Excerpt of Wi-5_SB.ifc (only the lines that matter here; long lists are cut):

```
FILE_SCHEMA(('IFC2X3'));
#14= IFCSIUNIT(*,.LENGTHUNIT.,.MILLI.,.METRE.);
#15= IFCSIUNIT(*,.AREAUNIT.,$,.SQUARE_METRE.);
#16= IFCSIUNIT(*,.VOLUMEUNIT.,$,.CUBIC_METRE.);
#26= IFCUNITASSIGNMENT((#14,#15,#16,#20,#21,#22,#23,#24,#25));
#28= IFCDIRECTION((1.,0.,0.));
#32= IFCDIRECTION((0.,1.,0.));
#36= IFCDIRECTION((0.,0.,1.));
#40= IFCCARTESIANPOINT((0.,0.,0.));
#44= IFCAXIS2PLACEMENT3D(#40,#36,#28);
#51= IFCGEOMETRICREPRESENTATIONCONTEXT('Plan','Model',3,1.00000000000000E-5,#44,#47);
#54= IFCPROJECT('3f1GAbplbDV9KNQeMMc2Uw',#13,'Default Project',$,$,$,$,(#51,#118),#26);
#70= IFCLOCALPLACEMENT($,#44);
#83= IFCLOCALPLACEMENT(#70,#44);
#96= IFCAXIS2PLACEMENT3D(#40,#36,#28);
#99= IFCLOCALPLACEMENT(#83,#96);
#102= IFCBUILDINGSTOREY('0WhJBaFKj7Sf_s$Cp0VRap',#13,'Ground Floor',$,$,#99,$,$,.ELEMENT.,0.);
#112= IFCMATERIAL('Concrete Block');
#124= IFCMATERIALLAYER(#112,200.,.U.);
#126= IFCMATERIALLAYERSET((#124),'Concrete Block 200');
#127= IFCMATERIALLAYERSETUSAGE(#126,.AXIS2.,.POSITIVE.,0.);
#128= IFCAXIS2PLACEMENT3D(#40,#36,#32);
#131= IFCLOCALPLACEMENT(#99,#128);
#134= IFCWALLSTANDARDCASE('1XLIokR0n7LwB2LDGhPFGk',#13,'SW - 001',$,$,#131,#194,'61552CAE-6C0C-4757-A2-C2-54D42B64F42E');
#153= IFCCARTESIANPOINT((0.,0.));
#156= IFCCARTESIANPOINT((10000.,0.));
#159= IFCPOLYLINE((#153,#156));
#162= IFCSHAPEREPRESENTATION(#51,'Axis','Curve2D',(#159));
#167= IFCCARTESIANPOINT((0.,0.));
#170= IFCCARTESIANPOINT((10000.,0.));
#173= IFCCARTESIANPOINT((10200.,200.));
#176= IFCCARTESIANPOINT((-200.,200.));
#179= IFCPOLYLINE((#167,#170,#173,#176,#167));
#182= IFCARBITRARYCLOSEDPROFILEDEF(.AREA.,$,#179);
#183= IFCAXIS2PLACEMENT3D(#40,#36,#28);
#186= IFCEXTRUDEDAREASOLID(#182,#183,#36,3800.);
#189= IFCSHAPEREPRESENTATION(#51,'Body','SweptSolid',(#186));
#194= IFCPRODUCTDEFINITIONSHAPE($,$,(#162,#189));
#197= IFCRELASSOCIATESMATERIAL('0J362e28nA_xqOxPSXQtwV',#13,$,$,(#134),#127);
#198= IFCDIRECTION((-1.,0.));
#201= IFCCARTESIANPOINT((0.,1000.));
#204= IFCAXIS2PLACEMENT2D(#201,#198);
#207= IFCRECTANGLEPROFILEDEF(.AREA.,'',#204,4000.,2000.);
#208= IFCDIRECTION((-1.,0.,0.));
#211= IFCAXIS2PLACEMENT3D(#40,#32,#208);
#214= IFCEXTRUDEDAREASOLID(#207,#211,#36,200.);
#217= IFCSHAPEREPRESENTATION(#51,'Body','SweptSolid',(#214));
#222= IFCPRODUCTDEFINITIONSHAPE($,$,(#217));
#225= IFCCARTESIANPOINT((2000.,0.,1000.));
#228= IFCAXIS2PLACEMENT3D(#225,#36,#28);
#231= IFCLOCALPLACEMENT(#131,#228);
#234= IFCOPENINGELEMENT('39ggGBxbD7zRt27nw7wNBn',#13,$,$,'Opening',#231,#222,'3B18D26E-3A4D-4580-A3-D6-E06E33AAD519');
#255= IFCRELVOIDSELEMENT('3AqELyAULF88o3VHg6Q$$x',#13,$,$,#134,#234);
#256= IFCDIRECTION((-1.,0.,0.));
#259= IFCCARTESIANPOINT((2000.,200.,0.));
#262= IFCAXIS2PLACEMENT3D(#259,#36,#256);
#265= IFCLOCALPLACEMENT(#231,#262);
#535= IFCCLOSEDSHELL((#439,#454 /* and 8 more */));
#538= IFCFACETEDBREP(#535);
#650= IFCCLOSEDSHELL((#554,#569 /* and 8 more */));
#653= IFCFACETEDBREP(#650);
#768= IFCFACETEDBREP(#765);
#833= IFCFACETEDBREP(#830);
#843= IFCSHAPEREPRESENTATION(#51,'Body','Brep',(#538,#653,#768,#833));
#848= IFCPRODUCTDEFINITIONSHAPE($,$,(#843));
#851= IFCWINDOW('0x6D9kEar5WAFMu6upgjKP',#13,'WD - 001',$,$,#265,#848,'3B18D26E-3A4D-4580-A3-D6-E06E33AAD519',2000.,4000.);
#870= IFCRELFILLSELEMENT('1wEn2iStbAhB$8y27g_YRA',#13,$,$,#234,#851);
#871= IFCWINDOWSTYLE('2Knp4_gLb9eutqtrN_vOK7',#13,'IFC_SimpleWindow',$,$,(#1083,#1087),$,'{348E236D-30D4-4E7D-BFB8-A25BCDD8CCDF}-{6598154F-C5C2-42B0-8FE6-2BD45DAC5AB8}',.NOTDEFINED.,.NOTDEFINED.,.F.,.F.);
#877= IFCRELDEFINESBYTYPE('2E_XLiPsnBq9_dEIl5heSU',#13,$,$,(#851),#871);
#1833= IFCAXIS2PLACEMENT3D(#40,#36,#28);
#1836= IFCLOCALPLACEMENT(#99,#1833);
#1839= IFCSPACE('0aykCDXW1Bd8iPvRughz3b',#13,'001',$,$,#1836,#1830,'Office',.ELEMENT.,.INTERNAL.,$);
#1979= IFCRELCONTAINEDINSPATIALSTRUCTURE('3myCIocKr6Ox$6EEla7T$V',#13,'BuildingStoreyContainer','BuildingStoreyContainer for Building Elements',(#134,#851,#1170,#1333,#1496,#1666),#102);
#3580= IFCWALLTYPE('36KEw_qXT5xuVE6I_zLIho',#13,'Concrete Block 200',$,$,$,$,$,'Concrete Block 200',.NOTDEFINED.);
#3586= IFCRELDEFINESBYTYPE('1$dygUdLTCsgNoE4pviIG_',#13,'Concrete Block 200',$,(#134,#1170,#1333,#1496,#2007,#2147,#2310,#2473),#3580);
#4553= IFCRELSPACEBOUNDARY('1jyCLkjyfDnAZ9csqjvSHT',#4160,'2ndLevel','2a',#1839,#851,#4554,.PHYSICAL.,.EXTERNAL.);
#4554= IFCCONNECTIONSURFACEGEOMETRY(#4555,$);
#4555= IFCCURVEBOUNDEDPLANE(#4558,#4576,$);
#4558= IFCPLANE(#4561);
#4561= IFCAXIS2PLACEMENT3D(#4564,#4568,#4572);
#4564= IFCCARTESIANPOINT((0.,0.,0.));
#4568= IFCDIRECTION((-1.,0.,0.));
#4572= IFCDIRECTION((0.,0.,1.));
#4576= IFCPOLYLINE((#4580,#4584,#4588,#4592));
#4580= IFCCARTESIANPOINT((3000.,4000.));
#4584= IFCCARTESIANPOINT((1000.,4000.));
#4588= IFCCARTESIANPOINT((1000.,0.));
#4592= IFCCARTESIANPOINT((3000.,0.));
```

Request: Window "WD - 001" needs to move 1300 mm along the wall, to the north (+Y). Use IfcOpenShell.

```python
import numpy as np
import ifcopenshell
import ifcopenshell.api.geometry
import ifcopenshell.util.placement

model = ifcopenshell.open("Wi-5_SB.ifc")

window = model.by_guid("0x6D9kEar5WAFMu6upgjKP")
opening = window.FillsVoids[0].RelatingOpeningElement
wall = opening.VoidsElements[0].RelatingBuildingElement

wall_matrix = ifcopenshell.util.placement.get_local_placement(wall.ObjectPlacement)
shift = wall_matrix[:3, 0] * 1300.0
before = ifcopenshell.util.placement.get_local_placement(window.ObjectPlacement)[:3, 3].copy()

# The window is placed relative to its opening, so it follows when the opening moves.
matrix = ifcopenshell.util.placement.get_local_placement(opening.ObjectPlacement)
matrix[:3, 3] += shift
ifcopenshell.api.geometry.edit_object_placement(
    model, product=opening, matrix=matrix, is_si=False, should_transform_children=True
)

# Space boundary surfaces are stored in each space's coordinates; move them too.
for rel in window.ProvidesBoundaries:
    if not rel.ConnectionGeometry:
        continue
    surface = rel.ConnectionGeometry.SurfaceOnRelatingElement.BasisSurface
    space_matrix = ifcopenshell.util.placement.get_local_placement(rel.RelatingSpace.ObjectPlacement)
    point = np.array(surface.Position.Location.Coordinates) + space_matrix[:3, :3].T @ shift
    surface.Position = model.createIfcAxis2Placement3D(
        model.createIfcCartesianPoint(point.tolist()), surface.Position.Axis, surface.Position.RefDirection
    )

after = ifcopenshell.util.placement.get_local_placement(window.ObjectPlacement)[:3, 3]
print("window moved by", (after - before).round(3) + 0.0)

model.write("Wi-5_SB_rev.ifc")
```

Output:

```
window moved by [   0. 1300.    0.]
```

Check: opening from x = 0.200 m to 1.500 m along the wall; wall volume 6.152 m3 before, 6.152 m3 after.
